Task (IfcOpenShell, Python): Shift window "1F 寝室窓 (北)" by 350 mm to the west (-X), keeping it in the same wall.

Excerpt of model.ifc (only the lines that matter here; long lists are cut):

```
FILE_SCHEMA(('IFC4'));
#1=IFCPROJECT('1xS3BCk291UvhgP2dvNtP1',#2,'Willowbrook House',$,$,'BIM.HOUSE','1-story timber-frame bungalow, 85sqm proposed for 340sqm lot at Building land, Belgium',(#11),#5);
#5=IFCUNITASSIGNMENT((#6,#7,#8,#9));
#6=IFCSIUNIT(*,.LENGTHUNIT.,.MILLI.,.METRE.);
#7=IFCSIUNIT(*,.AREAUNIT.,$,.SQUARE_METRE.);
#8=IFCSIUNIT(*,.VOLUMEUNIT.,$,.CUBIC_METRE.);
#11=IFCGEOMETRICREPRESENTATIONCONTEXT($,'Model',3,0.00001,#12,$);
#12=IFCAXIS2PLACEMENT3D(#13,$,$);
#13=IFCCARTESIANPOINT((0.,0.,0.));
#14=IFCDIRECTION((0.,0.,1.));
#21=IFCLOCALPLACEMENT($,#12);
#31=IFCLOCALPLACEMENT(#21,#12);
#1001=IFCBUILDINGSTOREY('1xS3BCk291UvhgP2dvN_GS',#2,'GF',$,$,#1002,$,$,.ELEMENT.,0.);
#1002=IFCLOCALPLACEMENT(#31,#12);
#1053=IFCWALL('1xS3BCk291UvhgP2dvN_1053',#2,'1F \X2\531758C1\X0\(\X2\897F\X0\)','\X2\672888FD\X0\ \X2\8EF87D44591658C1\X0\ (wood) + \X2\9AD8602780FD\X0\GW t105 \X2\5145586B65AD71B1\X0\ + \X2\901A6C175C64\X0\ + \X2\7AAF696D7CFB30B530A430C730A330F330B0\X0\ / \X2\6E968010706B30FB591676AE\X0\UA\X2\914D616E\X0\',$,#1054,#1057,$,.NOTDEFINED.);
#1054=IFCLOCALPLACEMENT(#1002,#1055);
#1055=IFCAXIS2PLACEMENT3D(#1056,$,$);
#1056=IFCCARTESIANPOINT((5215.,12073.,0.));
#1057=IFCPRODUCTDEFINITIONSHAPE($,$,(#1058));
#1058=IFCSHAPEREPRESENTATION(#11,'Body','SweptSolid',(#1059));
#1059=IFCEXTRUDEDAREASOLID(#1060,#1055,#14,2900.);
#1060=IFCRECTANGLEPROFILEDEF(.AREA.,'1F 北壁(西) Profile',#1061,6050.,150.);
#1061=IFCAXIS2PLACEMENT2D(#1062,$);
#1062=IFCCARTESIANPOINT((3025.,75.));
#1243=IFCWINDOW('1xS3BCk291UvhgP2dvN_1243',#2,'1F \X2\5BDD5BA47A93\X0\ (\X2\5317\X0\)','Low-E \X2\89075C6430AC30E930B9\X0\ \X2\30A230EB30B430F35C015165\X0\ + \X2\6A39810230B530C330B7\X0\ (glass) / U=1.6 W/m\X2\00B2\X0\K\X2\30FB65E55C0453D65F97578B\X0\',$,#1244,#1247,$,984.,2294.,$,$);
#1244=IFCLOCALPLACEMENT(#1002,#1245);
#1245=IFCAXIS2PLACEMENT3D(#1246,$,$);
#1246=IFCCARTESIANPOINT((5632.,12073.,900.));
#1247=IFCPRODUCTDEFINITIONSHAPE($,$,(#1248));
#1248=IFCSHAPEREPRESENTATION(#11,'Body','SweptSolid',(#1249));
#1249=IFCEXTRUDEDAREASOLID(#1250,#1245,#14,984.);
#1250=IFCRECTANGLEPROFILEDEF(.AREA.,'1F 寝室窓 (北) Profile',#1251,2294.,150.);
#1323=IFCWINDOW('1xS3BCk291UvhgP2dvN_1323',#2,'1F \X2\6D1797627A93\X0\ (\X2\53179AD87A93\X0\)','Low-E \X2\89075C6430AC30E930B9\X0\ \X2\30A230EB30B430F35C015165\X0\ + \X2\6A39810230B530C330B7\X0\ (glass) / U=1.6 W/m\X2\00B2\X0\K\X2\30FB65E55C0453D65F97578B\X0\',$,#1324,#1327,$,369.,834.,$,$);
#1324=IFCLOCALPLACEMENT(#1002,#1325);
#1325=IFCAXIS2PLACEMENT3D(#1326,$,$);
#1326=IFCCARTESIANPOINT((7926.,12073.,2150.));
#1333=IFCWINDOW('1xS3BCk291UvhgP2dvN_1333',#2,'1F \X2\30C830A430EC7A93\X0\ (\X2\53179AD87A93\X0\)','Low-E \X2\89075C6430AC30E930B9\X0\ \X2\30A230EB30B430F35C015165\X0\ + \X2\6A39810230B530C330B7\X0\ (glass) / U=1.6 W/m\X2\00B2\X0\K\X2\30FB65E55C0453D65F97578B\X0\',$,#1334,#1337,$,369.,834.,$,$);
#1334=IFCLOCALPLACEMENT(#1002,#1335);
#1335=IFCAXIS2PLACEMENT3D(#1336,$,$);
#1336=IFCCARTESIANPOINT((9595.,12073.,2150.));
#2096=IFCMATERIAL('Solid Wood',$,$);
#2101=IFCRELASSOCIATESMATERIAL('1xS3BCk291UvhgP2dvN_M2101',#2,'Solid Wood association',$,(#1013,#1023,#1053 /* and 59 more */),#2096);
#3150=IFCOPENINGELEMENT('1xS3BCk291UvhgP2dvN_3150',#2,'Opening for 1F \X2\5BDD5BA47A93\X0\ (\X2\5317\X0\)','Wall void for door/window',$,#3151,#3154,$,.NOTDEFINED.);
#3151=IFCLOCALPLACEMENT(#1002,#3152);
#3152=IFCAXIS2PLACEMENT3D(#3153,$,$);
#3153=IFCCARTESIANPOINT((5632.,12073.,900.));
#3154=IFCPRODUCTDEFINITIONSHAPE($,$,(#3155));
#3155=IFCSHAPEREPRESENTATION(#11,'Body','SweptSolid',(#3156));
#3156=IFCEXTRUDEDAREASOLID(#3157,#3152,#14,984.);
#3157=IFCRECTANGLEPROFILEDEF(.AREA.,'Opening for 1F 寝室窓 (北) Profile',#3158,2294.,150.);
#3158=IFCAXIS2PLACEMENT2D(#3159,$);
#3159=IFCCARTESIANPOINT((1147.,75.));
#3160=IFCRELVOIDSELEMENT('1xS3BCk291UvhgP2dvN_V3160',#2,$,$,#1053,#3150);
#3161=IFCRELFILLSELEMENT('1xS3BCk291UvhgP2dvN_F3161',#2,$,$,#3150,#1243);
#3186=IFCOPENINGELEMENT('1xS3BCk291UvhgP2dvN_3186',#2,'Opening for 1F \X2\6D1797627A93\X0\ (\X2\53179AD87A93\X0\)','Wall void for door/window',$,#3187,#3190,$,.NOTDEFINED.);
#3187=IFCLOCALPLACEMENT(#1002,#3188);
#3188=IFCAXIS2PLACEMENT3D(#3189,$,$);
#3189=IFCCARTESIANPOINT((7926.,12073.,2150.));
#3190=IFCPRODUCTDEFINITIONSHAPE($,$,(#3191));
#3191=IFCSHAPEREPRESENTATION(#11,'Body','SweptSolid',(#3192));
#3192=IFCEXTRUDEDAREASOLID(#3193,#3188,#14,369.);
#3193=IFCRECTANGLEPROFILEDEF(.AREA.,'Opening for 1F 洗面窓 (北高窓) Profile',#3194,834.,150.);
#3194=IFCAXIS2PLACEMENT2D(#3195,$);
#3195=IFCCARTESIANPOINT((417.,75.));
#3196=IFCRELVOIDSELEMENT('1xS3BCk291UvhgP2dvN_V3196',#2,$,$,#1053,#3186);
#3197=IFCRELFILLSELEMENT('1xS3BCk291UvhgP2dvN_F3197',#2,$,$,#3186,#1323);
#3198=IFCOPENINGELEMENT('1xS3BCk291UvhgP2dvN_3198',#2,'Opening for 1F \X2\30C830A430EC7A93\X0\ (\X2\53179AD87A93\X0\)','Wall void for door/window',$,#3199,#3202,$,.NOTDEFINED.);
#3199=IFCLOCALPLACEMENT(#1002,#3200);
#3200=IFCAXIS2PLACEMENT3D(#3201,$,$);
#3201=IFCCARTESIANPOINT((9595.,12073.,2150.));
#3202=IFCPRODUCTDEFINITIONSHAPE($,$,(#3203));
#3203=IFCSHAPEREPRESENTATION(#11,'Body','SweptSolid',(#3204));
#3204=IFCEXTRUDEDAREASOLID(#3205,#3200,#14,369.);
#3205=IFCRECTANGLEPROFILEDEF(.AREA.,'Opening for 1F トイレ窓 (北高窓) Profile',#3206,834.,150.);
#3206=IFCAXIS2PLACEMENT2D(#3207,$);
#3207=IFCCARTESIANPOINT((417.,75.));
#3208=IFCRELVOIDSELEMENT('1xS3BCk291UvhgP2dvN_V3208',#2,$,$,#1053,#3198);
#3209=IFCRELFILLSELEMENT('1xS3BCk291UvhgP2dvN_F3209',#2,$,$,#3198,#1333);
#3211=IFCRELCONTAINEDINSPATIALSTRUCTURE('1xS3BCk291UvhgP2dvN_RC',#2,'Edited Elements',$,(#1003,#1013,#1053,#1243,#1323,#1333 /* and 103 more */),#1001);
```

```python
import ifcopenshell
import ifcopenshell.api.geometry
import ifcopenshell.util.placement
import ifcopenshell.util.unit

model = ifcopenshell.open("model.ifc")
unit_scale = ifcopenshell.util.unit.calculate_unit_scale(model)

window = model.by_guid("1xS3BCk291UvhgP2dvN_1243")
opening = window.FillsVoids[0].RelatingOpeningElement
wall = opening.VoidsElements[0].RelatingBuildingElement

wall_matrix = ifcopenshell.util.placement.get_local_placement(wall.ObjectPlacement)
shift = wall_matrix[:3, 0] * -0.35 / unit_scale
before = ifcopenshell.util.placement.get_local_placement(window.ObjectPlacement)[:3, 3].copy()

# The window is not placed relative to its opening, so move both.
for product in (opening, window):
    matrix = ifcopenshell.util.placement.get_local_placement(product.ObjectPlacement)
    matrix[:3, 3] += shift
    ifcopenshell.api.geometry.edit_object_placement(model, product=product, matrix=matrix, is_si=False)

after = ifcopenshell.util.placement.get_local_placement(window.ObjectPlacement)[:3, 3]
print("window moved by", (after - before).round(3) + 0.0)

model.write("model-out.ifc")
```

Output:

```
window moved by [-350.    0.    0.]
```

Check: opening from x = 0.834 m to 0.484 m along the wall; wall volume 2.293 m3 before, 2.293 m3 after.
